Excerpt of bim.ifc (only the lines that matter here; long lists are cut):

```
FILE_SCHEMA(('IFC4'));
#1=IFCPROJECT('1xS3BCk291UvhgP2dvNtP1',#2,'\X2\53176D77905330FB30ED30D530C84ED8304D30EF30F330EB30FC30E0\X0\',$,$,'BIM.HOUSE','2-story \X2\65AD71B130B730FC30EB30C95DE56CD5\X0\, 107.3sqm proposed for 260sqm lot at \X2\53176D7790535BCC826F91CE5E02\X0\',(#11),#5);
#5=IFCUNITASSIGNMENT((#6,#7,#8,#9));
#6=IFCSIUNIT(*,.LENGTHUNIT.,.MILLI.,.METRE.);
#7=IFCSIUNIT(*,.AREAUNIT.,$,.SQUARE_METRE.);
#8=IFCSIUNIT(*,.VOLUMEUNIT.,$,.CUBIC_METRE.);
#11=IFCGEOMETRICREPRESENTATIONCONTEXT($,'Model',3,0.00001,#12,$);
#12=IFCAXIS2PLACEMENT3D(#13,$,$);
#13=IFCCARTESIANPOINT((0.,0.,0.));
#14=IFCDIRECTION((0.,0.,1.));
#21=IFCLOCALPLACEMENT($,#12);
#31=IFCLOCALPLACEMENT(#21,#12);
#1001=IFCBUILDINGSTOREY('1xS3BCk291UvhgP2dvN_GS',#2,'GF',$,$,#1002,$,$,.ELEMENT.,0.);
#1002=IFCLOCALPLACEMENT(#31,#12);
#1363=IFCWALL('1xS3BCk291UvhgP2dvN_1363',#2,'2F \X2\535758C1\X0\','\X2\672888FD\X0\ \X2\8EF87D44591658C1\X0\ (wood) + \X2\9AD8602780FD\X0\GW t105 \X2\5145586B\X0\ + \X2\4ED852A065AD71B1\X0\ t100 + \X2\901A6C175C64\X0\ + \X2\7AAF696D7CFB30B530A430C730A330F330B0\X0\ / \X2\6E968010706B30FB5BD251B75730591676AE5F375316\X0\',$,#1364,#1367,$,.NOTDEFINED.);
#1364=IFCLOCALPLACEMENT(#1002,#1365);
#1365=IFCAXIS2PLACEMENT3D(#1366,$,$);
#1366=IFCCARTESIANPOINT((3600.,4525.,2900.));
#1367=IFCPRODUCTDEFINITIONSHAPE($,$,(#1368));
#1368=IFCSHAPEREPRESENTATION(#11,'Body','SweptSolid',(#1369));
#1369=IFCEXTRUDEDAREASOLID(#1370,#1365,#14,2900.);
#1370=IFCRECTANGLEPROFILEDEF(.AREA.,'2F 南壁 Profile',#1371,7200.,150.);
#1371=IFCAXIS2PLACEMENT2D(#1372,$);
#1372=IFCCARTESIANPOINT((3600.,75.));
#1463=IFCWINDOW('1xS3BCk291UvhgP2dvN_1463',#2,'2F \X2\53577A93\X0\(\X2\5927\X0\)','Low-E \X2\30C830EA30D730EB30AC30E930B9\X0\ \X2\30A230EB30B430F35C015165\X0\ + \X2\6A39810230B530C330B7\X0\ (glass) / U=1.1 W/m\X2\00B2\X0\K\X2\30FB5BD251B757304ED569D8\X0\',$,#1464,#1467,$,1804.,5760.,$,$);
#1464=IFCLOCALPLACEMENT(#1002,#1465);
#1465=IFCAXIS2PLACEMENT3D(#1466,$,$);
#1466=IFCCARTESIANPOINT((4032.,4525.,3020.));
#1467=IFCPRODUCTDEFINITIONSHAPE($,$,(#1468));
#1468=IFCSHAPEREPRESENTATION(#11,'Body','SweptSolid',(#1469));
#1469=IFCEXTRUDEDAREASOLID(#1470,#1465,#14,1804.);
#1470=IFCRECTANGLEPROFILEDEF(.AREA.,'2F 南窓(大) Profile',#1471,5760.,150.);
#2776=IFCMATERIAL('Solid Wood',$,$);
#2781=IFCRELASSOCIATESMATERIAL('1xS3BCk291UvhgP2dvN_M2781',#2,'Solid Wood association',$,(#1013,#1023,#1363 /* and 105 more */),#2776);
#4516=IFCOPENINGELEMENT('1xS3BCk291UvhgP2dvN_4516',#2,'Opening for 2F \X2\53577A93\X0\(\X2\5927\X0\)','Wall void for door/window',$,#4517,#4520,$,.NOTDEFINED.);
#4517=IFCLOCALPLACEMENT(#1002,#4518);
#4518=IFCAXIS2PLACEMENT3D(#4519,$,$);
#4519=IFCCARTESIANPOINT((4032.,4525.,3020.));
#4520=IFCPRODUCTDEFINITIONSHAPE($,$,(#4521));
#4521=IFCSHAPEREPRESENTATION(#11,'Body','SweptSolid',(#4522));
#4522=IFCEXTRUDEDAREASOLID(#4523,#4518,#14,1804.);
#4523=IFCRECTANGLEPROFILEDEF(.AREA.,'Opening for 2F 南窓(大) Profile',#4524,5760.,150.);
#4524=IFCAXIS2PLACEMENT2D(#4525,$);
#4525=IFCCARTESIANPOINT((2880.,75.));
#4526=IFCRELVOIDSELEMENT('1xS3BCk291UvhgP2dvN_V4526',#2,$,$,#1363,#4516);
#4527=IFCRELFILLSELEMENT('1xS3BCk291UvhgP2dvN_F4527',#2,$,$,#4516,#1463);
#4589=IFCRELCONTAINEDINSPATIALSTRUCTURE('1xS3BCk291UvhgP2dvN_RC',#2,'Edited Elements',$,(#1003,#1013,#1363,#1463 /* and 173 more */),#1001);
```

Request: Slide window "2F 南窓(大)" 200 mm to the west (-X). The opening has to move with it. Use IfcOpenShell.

```python
import ifcopenshell
import ifcopenshell.api.geometry
import ifcopenshell.util.placement

model = ifcopenshell.open("bim.ifc")

window = model.by_id(1463)
opening = window.FillsVoids[0].RelatingOpeningElement
wall = opening.VoidsElements[0].RelatingBuildingElement

wall_matrix = ifcopenshell.util.placement.get_local_placement(wall.ObjectPlacement)
shift = wall_matrix[:3, 0] * -200.0
before = ifcopenshell.util.placement.get_local_placement(window.ObjectPlacement)[:3, 3].copy()

# The window is not placed relative to its opening, so move both.
for product in (opening, window):
    matrix = ifcopenshell.util.placement.get_local_placement(product.ObjectPlacement)
    matrix[:3, 3] += shift
    ifcopenshell.api.geometry.edit_object_placement(model, product=product, matrix=matrix, is_si=False)

after = ifcopenshell.util.placement.get_local_placement(window.ObjectPlacement)[:3, 3]
print("window moved by", (after - before).round(3) + 0.0)

model.write("bim_updated.ifc")
```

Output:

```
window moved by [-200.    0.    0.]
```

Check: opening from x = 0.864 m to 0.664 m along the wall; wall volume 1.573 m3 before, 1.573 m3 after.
